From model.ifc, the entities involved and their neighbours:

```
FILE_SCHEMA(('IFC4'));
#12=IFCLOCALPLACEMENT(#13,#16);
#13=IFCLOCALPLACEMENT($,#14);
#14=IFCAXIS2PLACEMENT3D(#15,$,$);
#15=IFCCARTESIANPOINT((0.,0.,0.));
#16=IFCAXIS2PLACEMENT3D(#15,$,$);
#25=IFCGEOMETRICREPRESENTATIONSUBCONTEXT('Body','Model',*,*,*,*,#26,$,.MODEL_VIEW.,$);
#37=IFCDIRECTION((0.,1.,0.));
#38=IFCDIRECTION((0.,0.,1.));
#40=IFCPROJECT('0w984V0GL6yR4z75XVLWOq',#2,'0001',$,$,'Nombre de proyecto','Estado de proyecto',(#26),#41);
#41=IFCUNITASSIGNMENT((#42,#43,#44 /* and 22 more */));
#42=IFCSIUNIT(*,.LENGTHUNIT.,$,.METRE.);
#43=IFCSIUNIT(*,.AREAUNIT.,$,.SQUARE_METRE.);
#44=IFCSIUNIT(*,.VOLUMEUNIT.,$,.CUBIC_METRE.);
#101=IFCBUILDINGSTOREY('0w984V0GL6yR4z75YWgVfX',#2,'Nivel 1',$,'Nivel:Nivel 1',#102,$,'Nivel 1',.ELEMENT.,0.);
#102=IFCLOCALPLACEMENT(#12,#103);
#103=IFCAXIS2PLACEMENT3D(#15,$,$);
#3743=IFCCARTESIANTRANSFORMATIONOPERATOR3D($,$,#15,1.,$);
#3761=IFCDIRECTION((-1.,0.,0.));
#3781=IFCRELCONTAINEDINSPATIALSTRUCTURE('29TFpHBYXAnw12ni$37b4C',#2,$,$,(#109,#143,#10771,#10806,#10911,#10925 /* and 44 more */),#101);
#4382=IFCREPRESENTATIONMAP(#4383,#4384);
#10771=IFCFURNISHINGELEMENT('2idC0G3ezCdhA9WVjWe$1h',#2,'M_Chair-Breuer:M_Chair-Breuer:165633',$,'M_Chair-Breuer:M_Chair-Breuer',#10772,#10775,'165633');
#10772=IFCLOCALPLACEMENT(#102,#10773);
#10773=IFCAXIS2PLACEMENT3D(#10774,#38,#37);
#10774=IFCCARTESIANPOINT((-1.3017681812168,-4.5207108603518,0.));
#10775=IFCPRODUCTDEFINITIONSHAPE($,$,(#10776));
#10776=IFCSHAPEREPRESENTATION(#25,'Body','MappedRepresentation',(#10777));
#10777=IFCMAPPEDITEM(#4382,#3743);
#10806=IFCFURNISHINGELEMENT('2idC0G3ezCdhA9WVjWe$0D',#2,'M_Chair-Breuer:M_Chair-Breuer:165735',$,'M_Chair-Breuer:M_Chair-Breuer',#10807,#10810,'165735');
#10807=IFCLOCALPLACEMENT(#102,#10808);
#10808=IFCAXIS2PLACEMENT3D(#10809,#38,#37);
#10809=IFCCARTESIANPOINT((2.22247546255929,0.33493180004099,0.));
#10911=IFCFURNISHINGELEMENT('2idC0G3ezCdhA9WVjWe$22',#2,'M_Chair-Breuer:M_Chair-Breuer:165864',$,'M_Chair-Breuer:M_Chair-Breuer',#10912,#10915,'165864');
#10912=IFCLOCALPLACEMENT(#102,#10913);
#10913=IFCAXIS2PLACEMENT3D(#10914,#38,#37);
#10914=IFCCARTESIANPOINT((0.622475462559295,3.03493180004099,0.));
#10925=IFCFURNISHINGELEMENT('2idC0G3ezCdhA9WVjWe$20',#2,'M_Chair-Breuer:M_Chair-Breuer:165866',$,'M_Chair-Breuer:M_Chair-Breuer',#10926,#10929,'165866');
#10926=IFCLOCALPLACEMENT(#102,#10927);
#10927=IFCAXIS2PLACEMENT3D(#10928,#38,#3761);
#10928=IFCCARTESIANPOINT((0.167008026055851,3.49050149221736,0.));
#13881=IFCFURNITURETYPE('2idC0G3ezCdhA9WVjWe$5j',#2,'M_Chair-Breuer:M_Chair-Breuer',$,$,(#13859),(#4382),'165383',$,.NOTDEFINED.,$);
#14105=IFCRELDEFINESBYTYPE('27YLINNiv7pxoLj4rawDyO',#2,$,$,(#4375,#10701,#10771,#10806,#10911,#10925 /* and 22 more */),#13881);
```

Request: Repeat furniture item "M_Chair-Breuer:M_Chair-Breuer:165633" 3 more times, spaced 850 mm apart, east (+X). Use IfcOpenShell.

```python
import numpy as np
import ifcopenshell
import ifcopenshell.api.geometry
import ifcopenshell.api.root
import ifcopenshell.util.element
import ifcopenshell.util.placement
import ifcopenshell.util.unit

model = ifcopenshell.open("model.ifc")
unit_scale = ifcopenshell.util.unit.calculate_unit_scale(model)


def reuse_history(source, copy):
    """copy_class also copies each property set's owner history, people and application; keep the originals."""
    for rel in copy.IsDefinedBy:
        if rel.is_a("IfcRelDefinesByProperties") and (history := rel.RelatingPropertyDefinition.OwnerHistory):
            rel.RelatingPropertyDefinition.OwnerHistory = source.OwnerHistory
            ifcopenshell.util.element.remove_deep2(model, history)


source = model.by_id(10771)
base = ifcopenshell.util.placement.get_local_placement(source.ObjectPlacement)
step = np.array([1.0, 0.0, 0.0]) * 0.85 / unit_scale

for i in range(1, 4):
    copy = ifcopenshell.api.root.copy_class(model, product=source)
    copy.Representation = ifcopenshell.util.element.copy_deep(
        model, source.Representation, exclude=["IfcGeometricRepresentationContext", "IfcRepresentationMap"]
    )
    copy.Name = "M_Chair-Breuer:M_Chair-Breuer"
    copy.Tag = None
    reuse_history(source, copy)
    matrix = base.copy()
    matrix[:3, 3] += i * step
    print("added at", matrix[:3, 3].round(3) + 0.0)
    ifcopenshell.api.geometry.edit_object_placement(model, product=copy, matrix=matrix, is_si=False)

model.write("model_updated.ifc")
```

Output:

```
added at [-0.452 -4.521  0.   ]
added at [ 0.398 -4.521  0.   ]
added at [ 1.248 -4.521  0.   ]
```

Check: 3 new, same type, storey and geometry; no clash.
